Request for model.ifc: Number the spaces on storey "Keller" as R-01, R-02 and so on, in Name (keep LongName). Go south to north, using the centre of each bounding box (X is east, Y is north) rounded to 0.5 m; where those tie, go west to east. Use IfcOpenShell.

First a look at what the model holds.

```python
import ifcopenshell
import ifcopenshell.util.element
import ifcopenshell.util.placement

model = ifcopenshell.open("model.ifc")
print(model.schema)
storey = next(s for s in model.by_type("IfcBuildingStorey") if s.Name == "Keller")
spaces = [e for e in ifcopenshell.util.element.get_decomposition(storey) if e.is_a("IfcSpace")]
for e in sorted(spaces, key=lambda e: e.id()):
    origin = ifcopenshell.util.placement.get_local_placement(e.ObjectPlacement)[:3, 3]
    print(e.id(), e.Name, e.LongName, origin.round(2) + 0.0, sep=" | ")
```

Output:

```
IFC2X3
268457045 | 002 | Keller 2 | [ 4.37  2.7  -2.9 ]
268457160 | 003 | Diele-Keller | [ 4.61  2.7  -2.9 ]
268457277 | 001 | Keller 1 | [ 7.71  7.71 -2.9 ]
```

```python
import ifcopenshell
import ifcopenshell.geom
import ifcopenshell.util.element
import ifcopenshell.util.shape

model = ifcopenshell.open("model.ifc")
settings = ifcopenshell.geom.settings()
settings.set("use-world-coords", True)


def centre(element):
    shape = ifcopenshell.geom.create_shape(settings, element)
    return ifcopenshell.util.shape.get_bbox_centroid(shape.geometry)


storey = next(s for s in model.by_type("IfcBuildingStorey") if s.Name == "Keller")
spaces = [e for e in ifcopenshell.util.element.get_decomposition(storey) if e.is_a("IfcSpace")]

# Insertion points can sit at a corner or the storey origin, so sort by the geometry (in metres).
centres = {e: centre(e) for e in spaces}
spaces.sort(key=lambda e: (round(centres[e][1] / 0.5), centres[e][0]))

for i, e in enumerate(spaces, start=1):
    number = f"R-{i:02d}"
    e.Name = number
    print(e.id(), number)

model.write("model_v2.ifc")
```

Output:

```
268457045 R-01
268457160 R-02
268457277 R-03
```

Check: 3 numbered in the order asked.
